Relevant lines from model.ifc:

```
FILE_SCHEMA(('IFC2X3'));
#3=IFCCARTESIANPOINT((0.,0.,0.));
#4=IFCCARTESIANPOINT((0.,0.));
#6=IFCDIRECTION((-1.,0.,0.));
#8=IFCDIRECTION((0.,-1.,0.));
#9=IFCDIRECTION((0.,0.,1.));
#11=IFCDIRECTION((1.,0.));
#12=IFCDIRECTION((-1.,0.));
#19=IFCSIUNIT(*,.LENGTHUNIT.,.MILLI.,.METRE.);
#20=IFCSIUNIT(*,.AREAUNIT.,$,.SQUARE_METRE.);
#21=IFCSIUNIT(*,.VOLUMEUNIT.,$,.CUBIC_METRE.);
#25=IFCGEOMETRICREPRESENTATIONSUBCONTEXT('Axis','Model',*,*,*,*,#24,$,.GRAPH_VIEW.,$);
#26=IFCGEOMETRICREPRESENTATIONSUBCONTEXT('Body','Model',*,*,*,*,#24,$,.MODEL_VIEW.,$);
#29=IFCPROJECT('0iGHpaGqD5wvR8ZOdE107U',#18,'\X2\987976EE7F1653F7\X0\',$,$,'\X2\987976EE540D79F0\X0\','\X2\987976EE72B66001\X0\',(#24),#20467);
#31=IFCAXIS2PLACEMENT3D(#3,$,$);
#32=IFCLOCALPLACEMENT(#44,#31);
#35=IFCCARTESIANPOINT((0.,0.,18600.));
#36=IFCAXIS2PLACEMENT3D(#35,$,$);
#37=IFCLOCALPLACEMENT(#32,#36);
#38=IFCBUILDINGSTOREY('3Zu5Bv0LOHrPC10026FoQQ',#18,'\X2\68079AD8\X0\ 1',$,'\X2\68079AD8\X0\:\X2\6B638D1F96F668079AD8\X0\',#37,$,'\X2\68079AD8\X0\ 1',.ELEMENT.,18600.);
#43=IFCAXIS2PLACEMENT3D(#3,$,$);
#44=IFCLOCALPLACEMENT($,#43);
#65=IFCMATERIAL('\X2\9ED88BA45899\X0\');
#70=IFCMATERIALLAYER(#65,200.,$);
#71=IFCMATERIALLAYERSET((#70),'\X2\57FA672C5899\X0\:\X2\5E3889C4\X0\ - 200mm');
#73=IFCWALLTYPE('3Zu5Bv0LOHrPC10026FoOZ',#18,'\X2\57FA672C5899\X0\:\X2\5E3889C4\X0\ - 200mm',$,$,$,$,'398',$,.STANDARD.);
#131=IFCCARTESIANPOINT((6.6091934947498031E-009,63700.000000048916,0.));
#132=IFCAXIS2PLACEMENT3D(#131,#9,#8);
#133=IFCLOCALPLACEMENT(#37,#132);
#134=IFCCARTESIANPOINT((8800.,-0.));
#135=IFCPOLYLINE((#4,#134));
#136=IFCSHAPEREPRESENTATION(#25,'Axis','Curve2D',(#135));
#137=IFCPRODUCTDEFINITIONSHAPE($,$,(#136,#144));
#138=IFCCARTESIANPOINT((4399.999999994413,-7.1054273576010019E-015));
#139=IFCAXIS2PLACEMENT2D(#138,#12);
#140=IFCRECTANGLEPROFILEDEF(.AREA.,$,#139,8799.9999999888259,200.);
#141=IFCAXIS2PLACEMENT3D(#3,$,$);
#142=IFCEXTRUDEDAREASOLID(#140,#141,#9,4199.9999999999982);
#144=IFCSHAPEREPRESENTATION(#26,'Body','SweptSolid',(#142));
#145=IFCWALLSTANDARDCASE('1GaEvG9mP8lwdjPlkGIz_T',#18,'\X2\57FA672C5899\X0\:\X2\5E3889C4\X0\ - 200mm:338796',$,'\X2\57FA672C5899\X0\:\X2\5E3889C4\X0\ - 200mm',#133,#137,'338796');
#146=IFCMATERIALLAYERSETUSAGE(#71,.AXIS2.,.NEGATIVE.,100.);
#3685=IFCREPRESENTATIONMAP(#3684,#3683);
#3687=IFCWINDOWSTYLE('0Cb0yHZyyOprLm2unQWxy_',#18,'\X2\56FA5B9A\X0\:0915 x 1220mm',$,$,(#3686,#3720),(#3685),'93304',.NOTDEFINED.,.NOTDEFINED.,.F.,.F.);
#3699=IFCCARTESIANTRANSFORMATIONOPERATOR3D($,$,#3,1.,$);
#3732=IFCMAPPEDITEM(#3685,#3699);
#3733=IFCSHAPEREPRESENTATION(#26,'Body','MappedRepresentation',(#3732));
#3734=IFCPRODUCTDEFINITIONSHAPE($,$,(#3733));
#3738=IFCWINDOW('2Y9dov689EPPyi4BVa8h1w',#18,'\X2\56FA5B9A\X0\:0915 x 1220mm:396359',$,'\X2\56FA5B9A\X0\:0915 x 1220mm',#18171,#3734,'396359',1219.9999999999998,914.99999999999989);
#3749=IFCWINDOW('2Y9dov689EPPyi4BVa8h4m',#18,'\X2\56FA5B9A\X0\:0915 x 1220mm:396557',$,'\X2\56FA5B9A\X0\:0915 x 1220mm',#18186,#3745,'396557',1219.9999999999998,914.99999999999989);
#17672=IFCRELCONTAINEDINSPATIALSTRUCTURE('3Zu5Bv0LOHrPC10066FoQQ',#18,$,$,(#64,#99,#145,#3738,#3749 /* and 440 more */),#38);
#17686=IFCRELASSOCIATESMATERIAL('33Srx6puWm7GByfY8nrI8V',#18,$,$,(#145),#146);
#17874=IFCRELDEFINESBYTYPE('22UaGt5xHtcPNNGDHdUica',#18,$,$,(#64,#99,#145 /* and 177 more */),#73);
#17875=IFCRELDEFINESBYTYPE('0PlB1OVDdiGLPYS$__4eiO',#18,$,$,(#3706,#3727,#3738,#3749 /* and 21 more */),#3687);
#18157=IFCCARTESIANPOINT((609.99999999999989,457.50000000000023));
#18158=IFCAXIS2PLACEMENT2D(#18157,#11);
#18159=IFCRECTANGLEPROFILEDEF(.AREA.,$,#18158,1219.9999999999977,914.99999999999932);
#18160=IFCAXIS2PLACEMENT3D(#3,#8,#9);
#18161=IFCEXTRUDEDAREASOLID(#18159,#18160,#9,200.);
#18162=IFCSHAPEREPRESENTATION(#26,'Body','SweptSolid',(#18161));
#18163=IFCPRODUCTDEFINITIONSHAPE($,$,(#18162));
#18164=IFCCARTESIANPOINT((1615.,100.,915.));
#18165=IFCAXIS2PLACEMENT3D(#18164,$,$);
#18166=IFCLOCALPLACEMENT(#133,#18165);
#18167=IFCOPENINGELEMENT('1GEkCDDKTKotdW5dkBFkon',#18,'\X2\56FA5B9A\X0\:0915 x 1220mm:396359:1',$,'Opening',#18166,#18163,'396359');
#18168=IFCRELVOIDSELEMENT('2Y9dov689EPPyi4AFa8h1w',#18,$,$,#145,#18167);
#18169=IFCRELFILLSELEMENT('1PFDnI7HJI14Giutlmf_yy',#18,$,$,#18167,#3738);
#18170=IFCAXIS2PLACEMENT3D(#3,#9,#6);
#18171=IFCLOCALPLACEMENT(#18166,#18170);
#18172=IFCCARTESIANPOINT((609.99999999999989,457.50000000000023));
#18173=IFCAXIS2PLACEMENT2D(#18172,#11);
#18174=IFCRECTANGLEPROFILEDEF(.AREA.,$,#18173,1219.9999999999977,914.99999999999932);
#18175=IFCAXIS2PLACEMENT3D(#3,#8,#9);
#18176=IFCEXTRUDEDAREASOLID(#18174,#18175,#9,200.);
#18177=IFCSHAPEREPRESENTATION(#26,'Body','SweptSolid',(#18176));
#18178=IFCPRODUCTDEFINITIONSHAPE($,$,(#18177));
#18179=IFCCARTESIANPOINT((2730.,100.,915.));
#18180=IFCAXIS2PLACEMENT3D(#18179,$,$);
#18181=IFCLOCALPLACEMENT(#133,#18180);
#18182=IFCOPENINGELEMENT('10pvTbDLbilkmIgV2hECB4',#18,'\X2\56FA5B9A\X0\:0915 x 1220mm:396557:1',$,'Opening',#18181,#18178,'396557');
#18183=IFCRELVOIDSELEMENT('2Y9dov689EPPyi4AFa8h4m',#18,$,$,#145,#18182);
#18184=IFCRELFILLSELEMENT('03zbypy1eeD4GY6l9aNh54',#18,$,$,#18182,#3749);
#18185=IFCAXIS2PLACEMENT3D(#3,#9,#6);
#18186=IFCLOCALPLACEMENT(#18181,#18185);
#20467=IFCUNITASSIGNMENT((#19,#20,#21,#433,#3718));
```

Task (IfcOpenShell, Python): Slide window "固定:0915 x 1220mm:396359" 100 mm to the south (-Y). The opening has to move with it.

```python
import ifcopenshell
import ifcopenshell.api.geometry
import ifcopenshell.util.placement
import ifcopenshell.util.unit

model = ifcopenshell.open("model.ifc")
unit_scale = ifcopenshell.util.unit.calculate_unit_scale(model)

window = model.by_id(3738)
opening = window.FillsVoids[0].RelatingOpeningElement
wall = opening.VoidsElements[0].RelatingBuildingElement

wall_matrix = ifcopenshell.util.placement.get_local_placement(wall.ObjectPlacement)
shift = wall_matrix[:3, 0] * 0.1 / unit_scale
before = ifcopenshell.util.placement.get_local_placement(window.ObjectPlacement)[:3, 3].copy()

# The window is placed relative to its opening, so it follows when the opening moves.
matrix = ifcopenshell.util.placement.get_local_placement(opening.ObjectPlacement)
matrix[:3, 3] += shift
ifcopenshell.api.geometry.edit_object_placement(
    model, product=opening, matrix=matrix, is_si=False, should_transform_children=True
)

after = ifcopenshell.util.placement.get_local_placement(window.ObjectPlacement)[:3, 3]
print("window moved by", (after - before).round(3) + 0.0)

model.write("model_v2.ifc")
```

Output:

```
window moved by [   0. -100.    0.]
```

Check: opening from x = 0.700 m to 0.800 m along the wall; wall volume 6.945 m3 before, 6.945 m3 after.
